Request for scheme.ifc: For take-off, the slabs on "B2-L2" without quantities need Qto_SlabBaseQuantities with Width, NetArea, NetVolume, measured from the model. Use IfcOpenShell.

First a look at what the model holds.

```python
import ifcopenshell
import ifcopenshell.util.element
import ifcopenshell.util.unit

model = ifcopenshell.open("scheme.ifc")
print(model.schema)
for unit_type in ("LENGTHUNIT", "AREAUNIT", "VOLUMEUNIT"):
    print(unit_type, ifcopenshell.util.unit.calculate_unit_scale(model, unit_type))
storey = next(s for s in model.by_type("IfcBuildingStorey") if s.Name == "B2-L2")
slabs = [e for e in ifcopenshell.util.element.get_decomposition(storey) if e.is_a("IfcSlab")]
for e in sorted(slabs, key=lambda e: e.id()):
    print(e.id(), e.is_a(), e.Name, list(ifcopenshell.util.element.get_psets(e, qtos_only=True)), sep=" | ")
```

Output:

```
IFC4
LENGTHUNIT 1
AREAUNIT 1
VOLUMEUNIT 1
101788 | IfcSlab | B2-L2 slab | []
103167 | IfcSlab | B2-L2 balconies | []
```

```python
import ifcopenshell
import ifcopenshell.api.pset
import ifcopenshell.geom
import ifcopenshell.util.element
import ifcopenshell.util.shape
import ifcopenshell.util.unit

model = ifcopenshell.open("scheme.ifc")
unit_scale = ifcopenshell.util.unit.calculate_unit_scale(model)
area_scale = ifcopenshell.util.unit.calculate_unit_scale(model, "AREAUNIT")
volume_scale = ifcopenshell.util.unit.calculate_unit_scale(model, "VOLUMEUNIT")
settings = ifcopenshell.geom.settings()

storey = next(s for s in model.by_type("IfcBuildingStorey") if s.Name == "B2-L2")
slabs = [e for e in ifcopenshell.util.element.get_decomposition(storey) if e.is_a("IfcSlab")]

for e in sorted(slabs, key=lambda e: e.id()):
    if ifcopenshell.util.element.get_psets(e, qtos_only=True, should_inherit=False):
        continue
    # Geometry comes back in metres, in the element's own axes.
    shape = ifcopenshell.geom.create_shape(settings, e)
    values = {
        "Width": ifcopenshell.util.shape.get_z(shape.geometry) / unit_scale,
        "NetArea": ifcopenshell.util.shape.get_footprint_area(shape.geometry) / area_scale,
        "NetVolume": ifcopenshell.util.shape.get_volume(shape.geometry) / volume_scale,
    }
    qto = ifcopenshell.api.pset.add_qto(model, product=e, name="Qto_SlabBaseQuantities")
    ifcopenshell.api.pset.edit_qto(model, qto=qto, properties=values)
    print(e.id(), {k: round(v, 3) for k, v in values.items()})

model.write("scheme_updated.ifc")
```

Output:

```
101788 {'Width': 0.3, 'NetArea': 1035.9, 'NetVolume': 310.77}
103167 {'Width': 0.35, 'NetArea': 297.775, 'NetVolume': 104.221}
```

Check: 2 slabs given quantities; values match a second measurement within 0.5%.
